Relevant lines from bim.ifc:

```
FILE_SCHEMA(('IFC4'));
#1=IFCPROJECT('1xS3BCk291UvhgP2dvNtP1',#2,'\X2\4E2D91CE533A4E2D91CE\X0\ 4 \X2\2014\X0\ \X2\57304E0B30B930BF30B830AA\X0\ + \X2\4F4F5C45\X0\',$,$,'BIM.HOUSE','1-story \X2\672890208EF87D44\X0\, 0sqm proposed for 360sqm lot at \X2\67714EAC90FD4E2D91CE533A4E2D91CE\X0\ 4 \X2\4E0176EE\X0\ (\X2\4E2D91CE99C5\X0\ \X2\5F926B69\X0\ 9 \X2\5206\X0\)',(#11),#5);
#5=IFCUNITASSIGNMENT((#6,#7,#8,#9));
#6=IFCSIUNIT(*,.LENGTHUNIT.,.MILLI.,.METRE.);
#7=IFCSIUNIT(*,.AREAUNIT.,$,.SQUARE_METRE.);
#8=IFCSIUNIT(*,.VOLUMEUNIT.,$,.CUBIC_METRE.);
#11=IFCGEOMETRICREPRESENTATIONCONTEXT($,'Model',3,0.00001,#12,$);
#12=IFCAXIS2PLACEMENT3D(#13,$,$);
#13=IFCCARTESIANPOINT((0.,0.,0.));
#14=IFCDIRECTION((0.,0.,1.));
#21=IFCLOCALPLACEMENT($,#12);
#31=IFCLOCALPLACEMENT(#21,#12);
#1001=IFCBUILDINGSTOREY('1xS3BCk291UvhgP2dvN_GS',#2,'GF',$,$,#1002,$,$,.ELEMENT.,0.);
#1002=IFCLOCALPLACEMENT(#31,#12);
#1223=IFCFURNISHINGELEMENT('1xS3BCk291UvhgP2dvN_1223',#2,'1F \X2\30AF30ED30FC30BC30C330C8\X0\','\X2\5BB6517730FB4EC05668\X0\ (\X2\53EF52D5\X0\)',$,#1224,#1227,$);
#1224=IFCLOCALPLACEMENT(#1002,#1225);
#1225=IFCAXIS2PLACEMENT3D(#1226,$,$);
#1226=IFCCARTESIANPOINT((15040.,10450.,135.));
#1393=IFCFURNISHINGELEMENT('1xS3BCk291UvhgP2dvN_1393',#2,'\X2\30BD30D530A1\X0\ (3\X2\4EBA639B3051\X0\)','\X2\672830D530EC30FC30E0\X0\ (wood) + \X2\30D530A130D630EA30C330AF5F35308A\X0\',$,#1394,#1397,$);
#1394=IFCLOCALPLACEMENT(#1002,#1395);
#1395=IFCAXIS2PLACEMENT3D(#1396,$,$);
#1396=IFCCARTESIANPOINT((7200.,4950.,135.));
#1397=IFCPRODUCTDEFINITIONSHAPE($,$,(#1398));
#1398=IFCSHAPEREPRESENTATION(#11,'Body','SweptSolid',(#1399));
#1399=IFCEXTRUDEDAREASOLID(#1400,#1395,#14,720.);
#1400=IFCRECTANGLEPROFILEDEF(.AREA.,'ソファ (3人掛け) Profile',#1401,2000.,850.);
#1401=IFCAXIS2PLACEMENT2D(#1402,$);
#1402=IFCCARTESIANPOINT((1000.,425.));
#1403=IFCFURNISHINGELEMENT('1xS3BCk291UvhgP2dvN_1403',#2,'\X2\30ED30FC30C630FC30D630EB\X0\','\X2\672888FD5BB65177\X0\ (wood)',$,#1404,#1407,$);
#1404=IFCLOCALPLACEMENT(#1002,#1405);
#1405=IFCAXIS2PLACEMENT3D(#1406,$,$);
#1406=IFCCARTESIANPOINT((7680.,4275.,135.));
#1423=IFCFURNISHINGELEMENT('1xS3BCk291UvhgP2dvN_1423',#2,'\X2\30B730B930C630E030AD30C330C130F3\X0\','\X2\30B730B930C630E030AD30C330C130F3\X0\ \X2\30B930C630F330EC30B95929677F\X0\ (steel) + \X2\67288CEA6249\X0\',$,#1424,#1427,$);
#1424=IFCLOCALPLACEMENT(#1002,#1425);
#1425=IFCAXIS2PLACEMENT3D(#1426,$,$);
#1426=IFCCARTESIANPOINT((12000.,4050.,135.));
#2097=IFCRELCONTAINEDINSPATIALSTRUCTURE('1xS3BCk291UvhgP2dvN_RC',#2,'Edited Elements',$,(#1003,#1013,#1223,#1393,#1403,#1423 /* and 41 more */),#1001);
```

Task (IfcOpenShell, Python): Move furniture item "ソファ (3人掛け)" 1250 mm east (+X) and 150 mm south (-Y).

```python
import ifcopenshell
import ifcopenshell.api.geometry
import ifcopenshell.util.placement
import ifcopenshell.util.unit

model = ifcopenshell.open("bim.ifc")
unit_scale = ifcopenshell.util.unit.calculate_unit_scale(model)

item = model.by_guid("1xS3BCk291UvhgP2dvN_1393")
matrix = ifcopenshell.util.placement.get_local_placement(item.ObjectPlacement)
matrix[0, 3] += 1.25 / unit_scale
matrix[1, 3] -= 0.15 / unit_scale
ifcopenshell.api.geometry.edit_object_placement(model, product=item, matrix=matrix, is_si=False)

print(ifcopenshell.util.placement.get_local_placement(item.ObjectPlacement).round(3) + 0.0)

model.write("bim-out.ifc")
```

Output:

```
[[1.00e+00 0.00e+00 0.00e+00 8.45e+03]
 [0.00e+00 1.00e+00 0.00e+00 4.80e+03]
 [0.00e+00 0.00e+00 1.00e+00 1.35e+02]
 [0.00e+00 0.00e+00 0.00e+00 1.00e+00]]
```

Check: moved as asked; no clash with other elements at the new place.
